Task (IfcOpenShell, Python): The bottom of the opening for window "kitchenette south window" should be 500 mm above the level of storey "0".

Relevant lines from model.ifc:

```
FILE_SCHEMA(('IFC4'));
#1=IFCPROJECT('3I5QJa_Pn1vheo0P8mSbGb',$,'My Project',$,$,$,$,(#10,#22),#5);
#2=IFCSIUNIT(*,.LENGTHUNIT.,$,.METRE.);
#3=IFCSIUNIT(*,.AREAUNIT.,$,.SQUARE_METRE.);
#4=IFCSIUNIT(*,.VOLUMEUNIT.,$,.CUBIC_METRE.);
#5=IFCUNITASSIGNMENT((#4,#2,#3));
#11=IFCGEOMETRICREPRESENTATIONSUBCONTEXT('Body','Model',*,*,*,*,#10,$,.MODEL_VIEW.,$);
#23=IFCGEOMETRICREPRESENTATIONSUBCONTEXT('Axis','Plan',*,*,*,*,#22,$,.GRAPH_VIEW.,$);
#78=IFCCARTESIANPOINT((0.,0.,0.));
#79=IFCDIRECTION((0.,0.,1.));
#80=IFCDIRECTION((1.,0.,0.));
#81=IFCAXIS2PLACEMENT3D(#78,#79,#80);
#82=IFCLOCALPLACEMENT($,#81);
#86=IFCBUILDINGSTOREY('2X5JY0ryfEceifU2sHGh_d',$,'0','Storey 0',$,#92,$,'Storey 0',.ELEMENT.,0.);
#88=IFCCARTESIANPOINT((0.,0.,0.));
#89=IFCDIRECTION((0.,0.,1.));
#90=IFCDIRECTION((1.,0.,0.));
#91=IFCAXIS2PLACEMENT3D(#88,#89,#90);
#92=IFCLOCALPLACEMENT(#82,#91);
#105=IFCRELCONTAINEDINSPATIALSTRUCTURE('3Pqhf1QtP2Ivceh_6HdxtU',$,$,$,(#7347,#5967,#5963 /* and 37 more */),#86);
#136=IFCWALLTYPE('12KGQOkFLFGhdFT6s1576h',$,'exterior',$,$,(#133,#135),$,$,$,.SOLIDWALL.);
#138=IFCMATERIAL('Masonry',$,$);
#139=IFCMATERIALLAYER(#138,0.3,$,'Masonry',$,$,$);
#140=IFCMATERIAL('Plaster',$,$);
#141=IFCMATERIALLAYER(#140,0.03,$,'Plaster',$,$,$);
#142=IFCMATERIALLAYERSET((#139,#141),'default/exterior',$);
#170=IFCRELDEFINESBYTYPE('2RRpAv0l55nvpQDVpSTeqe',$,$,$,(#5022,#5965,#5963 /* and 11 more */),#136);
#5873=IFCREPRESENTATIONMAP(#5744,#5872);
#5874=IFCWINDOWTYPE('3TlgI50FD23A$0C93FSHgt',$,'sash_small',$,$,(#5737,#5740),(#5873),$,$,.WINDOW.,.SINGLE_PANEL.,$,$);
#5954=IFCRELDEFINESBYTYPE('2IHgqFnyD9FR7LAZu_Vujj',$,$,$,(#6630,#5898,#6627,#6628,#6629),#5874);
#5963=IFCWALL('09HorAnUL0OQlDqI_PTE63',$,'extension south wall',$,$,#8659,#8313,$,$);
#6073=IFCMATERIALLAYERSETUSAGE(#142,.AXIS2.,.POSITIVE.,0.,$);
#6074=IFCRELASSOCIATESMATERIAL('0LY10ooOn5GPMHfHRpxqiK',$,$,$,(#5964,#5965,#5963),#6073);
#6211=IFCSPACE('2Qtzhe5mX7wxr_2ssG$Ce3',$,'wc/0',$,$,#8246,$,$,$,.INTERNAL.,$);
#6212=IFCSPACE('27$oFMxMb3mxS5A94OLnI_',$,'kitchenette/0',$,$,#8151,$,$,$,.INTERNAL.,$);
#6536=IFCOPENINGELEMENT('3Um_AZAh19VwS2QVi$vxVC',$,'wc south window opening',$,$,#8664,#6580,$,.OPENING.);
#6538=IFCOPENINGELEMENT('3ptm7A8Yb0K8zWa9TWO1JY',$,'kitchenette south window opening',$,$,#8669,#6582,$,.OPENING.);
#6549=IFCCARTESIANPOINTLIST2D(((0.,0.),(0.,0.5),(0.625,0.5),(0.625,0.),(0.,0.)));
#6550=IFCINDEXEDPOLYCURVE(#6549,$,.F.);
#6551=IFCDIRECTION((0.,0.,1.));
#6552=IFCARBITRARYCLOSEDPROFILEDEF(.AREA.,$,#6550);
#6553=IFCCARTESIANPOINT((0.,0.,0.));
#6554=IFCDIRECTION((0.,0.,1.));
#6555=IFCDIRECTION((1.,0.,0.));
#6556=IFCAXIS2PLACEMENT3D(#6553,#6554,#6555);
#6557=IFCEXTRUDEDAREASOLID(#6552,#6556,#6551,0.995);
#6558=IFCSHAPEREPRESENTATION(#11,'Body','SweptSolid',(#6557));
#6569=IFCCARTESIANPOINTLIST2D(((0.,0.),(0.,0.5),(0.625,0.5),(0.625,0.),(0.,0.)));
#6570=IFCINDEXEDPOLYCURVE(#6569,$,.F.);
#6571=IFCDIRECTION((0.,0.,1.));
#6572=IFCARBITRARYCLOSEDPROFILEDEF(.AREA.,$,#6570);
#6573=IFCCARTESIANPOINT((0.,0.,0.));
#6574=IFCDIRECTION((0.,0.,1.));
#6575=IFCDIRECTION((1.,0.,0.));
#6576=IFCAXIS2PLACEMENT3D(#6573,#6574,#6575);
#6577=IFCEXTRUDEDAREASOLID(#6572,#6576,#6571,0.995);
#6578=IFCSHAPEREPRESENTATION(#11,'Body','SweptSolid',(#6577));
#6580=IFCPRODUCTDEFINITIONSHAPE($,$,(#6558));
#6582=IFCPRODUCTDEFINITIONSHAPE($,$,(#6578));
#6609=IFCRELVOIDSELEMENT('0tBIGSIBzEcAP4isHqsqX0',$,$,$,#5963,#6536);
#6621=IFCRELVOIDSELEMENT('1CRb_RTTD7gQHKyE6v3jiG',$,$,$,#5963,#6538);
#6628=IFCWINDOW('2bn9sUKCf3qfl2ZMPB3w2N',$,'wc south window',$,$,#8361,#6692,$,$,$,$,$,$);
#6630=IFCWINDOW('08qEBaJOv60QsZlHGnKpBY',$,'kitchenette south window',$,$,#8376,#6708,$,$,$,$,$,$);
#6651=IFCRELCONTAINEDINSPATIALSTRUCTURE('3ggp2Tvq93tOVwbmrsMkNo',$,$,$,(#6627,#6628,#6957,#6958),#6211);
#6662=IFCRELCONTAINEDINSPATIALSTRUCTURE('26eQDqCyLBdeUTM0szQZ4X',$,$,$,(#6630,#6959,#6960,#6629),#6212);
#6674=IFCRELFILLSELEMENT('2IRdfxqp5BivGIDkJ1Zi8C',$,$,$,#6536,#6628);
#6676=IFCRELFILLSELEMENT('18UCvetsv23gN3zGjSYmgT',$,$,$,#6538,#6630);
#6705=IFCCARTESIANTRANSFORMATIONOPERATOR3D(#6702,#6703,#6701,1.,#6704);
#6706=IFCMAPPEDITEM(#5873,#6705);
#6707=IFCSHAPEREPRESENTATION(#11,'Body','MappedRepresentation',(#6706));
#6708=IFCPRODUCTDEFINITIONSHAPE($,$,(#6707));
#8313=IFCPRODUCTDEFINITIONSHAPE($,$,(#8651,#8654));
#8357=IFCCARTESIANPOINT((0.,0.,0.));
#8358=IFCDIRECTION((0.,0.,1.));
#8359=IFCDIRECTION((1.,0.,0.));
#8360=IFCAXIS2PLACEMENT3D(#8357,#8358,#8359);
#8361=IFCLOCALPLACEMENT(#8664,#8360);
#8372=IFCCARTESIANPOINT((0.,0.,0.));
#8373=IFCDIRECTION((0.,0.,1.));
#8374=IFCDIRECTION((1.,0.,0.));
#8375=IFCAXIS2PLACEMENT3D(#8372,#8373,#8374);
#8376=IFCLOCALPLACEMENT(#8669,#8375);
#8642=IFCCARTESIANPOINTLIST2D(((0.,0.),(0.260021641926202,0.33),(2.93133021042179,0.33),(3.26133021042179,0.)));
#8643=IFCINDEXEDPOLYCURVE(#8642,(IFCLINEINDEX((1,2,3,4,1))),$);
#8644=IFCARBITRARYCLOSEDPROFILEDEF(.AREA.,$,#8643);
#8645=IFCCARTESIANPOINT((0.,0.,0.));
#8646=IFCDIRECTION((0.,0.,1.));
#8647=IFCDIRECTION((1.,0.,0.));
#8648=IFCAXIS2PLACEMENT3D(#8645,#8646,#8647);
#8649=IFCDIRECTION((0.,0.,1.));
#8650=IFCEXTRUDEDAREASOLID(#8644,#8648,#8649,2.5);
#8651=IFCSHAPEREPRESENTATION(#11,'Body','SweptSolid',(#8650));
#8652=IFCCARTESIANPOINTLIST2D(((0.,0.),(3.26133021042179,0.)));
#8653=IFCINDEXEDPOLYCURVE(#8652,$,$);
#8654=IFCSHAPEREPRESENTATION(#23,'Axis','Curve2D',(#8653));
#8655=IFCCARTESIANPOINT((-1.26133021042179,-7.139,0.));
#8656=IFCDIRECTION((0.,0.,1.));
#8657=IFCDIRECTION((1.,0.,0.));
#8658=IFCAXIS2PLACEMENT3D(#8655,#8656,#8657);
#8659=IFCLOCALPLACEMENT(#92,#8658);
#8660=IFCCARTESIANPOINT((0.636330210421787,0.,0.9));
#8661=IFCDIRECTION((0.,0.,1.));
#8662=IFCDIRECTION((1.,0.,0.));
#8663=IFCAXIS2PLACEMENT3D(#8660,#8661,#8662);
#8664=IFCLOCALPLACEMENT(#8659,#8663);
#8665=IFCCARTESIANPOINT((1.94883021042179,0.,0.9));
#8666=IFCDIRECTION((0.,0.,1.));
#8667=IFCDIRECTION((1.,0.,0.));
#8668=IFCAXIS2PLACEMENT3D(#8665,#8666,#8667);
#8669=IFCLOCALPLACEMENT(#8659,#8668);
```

```python
import numpy as np
import ifcopenshell
import ifcopenshell.api.geometry
import ifcopenshell.geom
import ifcopenshell.util.element
import ifcopenshell.util.placement
import ifcopenshell.util.shape
import ifcopenshell.util.unit

model = ifcopenshell.open("model.ifc")
unit_scale = ifcopenshell.util.unit.calculate_unit_scale(model)

window = model.by_guid("08qEBaJOv60QsZlHGnKpBY")
opening = window.FillsVoids[0].RelatingOpeningElement
storey = ifcopenshell.util.element.get_container(window, ifc_class="IfcBuildingStorey")
level = ifcopenshell.util.placement.get_local_placement(storey.ObjectPlacement)[2, 3]

# The opening's origin need not be at the sill, so measure its lowest point.
shape = ifcopenshell.geom.create_shape(ifcopenshell.geom.settings(), opening)
bottom = ifcopenshell.util.shape.get_shape_bottom_elevation(shape, shape.geometry) / unit_scale
dz = level + 0.5 / unit_scale - bottom

shift = np.array([0.0, 0.0, dz])
# The window is placed relative to its opening, so it follows when the opening moves.
matrix = ifcopenshell.util.placement.get_local_placement(opening.ObjectPlacement)
matrix[:3, 3] += shift
ifcopenshell.api.geometry.edit_object_placement(
    model, product=opening, matrix=matrix, is_si=False, should_transform_children=True
)

print(f"moved by {dz * unit_scale:+.3f} m")

model.write("model_rev.ifc")
```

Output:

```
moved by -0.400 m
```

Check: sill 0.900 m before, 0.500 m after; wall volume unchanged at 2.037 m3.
